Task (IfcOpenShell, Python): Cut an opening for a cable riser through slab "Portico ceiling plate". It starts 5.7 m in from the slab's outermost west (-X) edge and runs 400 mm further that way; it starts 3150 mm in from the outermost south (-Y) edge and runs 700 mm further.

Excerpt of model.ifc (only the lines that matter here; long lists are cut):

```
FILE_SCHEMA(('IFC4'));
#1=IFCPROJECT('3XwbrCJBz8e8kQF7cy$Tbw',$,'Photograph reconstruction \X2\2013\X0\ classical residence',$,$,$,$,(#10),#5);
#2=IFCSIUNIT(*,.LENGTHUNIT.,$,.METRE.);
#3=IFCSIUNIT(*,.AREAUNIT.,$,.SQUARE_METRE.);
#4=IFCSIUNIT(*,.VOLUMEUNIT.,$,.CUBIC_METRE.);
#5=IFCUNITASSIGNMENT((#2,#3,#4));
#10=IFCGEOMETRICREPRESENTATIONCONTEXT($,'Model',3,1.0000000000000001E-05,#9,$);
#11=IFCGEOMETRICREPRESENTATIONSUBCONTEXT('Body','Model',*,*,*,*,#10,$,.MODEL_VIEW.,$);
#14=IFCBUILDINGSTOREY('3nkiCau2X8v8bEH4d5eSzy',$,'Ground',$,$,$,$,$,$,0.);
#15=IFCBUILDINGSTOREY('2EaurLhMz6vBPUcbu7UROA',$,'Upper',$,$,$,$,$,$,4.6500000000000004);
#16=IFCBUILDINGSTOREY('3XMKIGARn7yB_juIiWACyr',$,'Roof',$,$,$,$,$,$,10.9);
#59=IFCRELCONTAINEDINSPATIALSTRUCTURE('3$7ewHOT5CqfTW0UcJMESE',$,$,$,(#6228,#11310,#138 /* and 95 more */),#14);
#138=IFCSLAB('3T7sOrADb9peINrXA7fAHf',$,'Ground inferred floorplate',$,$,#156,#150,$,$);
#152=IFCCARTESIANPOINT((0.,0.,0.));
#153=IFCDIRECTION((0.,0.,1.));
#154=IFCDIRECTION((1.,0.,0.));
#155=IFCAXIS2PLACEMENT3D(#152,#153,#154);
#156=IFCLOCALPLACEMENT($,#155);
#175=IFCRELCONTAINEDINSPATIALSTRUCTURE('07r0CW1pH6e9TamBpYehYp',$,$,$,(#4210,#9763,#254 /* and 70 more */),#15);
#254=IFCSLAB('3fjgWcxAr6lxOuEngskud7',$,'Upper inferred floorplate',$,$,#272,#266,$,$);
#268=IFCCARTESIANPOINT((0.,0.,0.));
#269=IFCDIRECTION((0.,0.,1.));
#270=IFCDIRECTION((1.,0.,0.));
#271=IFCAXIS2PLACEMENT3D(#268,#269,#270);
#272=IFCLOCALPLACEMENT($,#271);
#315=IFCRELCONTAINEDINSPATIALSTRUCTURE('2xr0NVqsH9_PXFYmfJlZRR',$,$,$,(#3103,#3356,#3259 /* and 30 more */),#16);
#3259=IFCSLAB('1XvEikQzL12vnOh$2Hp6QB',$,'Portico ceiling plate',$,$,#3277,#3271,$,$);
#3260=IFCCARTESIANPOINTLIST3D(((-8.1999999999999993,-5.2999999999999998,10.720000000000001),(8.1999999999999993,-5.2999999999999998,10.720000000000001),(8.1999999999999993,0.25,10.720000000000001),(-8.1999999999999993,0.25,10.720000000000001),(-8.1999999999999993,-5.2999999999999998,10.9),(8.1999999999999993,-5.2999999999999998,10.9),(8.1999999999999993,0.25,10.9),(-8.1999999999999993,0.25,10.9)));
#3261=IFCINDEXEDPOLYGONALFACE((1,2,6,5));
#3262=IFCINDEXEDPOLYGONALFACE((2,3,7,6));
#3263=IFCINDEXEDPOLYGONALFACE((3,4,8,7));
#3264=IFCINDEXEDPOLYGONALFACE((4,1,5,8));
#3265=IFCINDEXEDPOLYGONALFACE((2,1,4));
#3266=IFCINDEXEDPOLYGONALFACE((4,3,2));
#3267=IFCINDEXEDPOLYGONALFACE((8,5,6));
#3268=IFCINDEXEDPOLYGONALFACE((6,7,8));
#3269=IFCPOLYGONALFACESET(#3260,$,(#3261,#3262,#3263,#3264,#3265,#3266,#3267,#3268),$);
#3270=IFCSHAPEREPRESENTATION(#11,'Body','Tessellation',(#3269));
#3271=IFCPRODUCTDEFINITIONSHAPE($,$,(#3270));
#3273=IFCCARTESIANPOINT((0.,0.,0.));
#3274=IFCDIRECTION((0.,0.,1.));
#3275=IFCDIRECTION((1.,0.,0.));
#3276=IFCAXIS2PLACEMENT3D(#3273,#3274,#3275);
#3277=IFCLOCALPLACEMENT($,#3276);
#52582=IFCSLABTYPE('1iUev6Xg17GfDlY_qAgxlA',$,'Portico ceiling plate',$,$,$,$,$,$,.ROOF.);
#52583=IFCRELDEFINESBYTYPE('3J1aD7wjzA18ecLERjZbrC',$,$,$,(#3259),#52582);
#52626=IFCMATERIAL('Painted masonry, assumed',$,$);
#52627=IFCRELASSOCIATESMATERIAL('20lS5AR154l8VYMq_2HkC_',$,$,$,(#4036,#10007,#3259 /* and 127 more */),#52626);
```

```python
import numpy as np
import ifcopenshell
import ifcopenshell.api.feature
import ifcopenshell.api.geometry
import ifcopenshell.api.root
import ifcopenshell.geom
import ifcopenshell.util.placement
import ifcopenshell.util.representation
import ifcopenshell.util.shape
import ifcopenshell.util.unit

model = ifcopenshell.open("model.ifc")
unit_scale = ifcopenshell.util.unit.calculate_unit_scale(model)
settings = ifcopenshell.geom.settings()


def volume(element):
    """Net volume in cubic metres, openings subtracted."""
    shape = ifcopenshell.geom.create_shape(settings, element)
    return ifcopenshell.util.shape.get_volume(shape.geometry)


slab = model.by_guid("1XvEikQzL12vnOh$2Hp6QB")
before = volume(slab)

# Extent in the slab's own axes, in metres. The edges named are its -X and -Y sides.
slab_shape = ifcopenshell.geom.create_shape(settings, slab)
vertices = ifcopenshell.util.shape.get_vertices(slab_shape.geometry)
x_min, y_min, bottom = vertices.min(axis=0)
top = vertices[:, 2].max()

opening = ifcopenshell.api.root.create_entity(model, ifc_class="IfcOpeningElement", name="Cable riser opening", predefined_type="OPENING")
context = ifcopenshell.util.representation.get_context(model, "Model", "Body", "MODEL_VIEW")
width, depth = 0.4, 0.7
outline = [(0.0, 0.0), (width, 0.0), (width, depth), (0.0, depth), (0.0, 0.0)]
# Overshoot both faces by 50 mm so the cut is clean.
shape = ifcopenshell.api.geometry.add_slab_representation(
    model, context=context, depth=top - bottom + 0.1, polyline=outline
)
ifcopenshell.api.geometry.assign_representation(model, product=opening, representation=shape)

matrix = ifcopenshell.util.placement.get_local_placement(slab.ObjectPlacement)
matrix[:, 3] = matrix @ np.append(np.array([x_min + 5.7, y_min + 3.15, bottom - 0.05]) / unit_scale, 1.0)
ifcopenshell.api.geometry.edit_object_placement(model, product=opening, matrix=matrix, is_si=False)
ifcopenshell.api.feature.add_feature(model, feature=opening, element=slab)

after = volume(slab)

print(f"slab volume {before:.3f} -> {after:.3f} m3")

model.write("model_updated.ifc")
```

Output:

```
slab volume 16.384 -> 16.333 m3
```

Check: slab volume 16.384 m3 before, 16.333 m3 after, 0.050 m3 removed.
